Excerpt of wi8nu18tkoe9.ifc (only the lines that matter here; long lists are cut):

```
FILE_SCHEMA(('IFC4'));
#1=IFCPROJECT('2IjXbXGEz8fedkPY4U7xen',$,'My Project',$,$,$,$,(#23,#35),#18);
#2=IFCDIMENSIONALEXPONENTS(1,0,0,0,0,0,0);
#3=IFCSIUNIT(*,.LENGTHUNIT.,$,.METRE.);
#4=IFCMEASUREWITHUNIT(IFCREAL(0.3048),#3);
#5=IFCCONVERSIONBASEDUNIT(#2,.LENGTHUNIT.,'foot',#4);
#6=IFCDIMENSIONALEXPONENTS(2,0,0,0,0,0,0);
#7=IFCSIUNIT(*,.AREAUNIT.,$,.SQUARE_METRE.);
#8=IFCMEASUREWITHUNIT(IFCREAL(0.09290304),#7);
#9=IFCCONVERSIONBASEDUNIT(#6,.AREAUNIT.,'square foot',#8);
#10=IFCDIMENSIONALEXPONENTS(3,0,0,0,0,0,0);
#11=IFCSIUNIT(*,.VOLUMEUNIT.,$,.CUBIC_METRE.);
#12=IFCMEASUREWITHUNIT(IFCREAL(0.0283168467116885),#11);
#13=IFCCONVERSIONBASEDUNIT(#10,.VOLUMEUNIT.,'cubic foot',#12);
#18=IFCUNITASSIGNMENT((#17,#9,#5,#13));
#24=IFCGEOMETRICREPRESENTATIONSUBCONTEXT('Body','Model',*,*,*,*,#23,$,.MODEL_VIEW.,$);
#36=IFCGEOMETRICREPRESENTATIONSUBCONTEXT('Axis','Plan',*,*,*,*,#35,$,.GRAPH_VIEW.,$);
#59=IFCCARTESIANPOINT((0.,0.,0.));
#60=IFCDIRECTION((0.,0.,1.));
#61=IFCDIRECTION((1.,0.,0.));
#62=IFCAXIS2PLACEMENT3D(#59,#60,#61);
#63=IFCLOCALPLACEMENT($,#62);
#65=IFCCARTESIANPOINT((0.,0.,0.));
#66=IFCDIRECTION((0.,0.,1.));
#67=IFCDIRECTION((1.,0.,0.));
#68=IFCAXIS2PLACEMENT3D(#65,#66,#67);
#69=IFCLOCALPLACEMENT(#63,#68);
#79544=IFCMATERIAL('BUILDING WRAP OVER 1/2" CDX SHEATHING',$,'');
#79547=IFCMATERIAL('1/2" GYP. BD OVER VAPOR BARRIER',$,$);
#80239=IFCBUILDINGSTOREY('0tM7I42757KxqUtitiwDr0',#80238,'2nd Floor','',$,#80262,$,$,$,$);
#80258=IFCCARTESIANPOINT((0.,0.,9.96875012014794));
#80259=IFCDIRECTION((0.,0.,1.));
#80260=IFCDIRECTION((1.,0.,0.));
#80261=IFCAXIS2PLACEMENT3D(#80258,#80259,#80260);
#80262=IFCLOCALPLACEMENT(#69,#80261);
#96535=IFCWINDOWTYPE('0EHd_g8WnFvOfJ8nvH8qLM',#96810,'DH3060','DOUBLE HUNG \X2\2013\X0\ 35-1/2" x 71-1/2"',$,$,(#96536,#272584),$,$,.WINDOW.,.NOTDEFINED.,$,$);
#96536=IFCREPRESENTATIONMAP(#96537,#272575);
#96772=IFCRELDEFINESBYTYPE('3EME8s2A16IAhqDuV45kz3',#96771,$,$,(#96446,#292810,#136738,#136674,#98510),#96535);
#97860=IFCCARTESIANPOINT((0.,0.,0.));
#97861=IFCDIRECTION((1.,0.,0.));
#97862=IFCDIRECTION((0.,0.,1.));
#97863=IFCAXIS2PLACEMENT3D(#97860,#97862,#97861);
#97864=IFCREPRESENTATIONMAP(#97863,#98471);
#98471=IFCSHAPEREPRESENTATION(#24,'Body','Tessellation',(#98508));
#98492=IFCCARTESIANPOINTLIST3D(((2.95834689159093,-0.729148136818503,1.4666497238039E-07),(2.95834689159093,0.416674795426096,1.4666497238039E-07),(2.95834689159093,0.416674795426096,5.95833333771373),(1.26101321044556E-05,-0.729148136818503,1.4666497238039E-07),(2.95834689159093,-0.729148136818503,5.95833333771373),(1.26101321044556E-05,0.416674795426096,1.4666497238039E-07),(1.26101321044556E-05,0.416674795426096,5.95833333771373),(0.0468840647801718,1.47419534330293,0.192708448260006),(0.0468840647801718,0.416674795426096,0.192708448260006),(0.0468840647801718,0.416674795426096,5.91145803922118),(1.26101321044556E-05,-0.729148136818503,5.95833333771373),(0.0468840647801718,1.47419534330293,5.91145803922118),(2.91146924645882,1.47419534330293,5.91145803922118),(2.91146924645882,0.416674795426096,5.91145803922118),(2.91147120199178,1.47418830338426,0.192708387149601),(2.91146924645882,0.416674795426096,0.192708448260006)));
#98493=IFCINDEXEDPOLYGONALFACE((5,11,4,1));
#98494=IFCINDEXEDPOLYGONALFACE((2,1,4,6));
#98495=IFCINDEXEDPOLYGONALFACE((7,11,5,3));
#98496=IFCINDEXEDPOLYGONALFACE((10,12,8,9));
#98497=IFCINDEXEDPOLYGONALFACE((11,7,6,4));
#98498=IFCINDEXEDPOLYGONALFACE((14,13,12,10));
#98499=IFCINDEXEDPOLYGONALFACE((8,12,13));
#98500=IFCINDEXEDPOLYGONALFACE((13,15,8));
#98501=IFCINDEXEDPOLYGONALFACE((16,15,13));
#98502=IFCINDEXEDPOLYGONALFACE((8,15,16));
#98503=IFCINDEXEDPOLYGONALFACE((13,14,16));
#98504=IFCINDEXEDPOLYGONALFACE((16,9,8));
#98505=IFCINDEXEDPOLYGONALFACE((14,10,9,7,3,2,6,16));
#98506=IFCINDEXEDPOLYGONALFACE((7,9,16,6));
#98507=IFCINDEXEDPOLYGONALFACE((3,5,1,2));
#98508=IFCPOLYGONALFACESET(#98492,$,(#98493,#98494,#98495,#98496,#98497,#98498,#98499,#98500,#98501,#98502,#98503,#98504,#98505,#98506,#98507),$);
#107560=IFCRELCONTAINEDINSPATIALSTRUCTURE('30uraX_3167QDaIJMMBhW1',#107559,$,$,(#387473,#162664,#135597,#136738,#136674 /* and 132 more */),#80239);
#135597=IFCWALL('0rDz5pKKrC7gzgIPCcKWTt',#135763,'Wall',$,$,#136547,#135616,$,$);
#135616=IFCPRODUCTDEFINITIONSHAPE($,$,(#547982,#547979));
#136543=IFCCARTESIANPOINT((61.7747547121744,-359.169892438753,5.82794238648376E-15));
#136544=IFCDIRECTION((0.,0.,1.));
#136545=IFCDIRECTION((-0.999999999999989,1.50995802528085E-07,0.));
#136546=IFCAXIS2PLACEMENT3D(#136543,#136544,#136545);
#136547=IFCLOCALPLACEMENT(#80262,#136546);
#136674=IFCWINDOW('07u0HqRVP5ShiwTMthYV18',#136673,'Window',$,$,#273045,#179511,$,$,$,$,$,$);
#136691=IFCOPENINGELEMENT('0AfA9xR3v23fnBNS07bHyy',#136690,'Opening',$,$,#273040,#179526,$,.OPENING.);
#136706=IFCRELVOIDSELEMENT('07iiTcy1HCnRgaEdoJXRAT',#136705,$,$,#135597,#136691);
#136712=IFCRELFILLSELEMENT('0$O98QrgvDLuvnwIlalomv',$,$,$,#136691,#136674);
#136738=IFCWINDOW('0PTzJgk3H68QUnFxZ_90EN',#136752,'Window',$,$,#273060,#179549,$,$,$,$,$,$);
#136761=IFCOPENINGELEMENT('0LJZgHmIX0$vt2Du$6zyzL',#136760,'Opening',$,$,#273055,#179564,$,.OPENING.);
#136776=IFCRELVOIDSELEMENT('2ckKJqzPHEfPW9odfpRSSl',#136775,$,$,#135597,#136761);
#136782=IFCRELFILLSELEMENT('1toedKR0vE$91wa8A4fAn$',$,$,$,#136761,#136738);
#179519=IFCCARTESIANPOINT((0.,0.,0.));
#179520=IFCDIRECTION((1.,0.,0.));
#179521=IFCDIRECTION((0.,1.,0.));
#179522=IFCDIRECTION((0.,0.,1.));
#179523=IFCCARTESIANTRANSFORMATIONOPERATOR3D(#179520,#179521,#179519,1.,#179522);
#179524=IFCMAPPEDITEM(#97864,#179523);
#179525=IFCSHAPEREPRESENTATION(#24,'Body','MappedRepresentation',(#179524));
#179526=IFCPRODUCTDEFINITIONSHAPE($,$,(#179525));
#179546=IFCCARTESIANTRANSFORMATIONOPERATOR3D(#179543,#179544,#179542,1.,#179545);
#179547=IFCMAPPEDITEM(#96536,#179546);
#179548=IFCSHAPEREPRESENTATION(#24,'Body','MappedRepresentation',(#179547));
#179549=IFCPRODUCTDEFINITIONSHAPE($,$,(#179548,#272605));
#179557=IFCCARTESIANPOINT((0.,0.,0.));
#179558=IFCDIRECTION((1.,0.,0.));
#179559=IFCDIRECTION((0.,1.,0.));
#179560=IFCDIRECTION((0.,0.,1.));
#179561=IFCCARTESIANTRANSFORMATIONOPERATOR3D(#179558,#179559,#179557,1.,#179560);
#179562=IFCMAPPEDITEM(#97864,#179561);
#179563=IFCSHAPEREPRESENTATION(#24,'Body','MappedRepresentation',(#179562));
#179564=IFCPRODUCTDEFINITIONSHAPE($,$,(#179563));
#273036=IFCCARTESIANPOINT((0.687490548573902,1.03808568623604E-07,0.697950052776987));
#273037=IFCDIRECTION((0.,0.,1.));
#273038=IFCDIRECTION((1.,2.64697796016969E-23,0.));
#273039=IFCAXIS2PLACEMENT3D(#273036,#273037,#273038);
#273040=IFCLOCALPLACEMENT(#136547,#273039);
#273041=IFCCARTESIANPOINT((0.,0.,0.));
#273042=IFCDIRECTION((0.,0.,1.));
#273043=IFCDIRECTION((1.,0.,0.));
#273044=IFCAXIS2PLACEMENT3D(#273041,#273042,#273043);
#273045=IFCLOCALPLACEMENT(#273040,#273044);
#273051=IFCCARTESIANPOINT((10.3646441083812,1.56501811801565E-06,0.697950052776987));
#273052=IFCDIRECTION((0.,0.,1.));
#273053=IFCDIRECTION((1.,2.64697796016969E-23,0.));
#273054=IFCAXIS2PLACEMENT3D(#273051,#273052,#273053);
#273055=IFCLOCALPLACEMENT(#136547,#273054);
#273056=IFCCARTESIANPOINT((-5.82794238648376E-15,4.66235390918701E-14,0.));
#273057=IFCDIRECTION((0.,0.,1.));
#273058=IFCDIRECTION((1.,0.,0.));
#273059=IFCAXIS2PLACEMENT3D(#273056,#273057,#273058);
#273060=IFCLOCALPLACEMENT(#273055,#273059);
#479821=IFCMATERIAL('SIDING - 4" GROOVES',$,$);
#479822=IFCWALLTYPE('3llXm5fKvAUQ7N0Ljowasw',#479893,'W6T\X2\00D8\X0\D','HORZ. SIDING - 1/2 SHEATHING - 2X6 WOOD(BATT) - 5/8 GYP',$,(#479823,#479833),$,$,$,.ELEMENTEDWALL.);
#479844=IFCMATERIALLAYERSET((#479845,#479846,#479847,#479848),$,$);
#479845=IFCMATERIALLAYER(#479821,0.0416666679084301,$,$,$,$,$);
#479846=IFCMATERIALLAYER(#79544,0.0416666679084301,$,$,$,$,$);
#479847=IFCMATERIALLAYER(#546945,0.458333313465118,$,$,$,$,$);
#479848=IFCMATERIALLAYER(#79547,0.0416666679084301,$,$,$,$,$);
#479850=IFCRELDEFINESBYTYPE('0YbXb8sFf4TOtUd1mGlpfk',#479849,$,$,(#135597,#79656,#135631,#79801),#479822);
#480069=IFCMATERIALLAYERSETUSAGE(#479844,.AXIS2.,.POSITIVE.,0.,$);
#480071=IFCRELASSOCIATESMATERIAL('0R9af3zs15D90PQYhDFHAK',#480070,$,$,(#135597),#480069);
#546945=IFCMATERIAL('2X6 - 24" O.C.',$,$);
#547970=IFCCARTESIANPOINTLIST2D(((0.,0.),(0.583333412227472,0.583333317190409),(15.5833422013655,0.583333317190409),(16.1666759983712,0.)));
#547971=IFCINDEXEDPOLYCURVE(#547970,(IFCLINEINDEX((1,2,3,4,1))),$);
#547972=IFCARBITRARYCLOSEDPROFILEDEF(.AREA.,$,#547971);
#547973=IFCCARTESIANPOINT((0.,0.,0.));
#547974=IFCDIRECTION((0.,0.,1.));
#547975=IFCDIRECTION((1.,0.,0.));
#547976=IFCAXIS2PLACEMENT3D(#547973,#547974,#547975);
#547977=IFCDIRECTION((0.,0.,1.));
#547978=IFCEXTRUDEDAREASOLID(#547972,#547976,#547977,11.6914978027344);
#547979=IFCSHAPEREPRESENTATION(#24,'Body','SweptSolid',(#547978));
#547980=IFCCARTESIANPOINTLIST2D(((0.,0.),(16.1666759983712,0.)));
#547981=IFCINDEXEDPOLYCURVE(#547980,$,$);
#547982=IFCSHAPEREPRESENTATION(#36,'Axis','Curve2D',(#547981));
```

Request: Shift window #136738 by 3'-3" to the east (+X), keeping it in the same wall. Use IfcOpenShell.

```python
import ifcopenshell
import ifcopenshell.api.geometry
import ifcopenshell.util.placement
import ifcopenshell.util.unit

model = ifcopenshell.open("wi8nu18tkoe9.ifc")
unit_scale = ifcopenshell.util.unit.calculate_unit_scale(model)

window = model.by_id(136738)
opening = window.FillsVoids[0].RelatingOpeningElement
wall = opening.VoidsElements[0].RelatingBuildingElement

wall_matrix = ifcopenshell.util.placement.get_local_placement(wall.ObjectPlacement)
shift = wall_matrix[:3, 0] * -39 * 0.0254 / unit_scale
before = ifcopenshell.util.placement.get_local_placement(window.ObjectPlacement)[:3, 3].copy()

# The window is placed relative to its opening, so it follows when the opening moves.
matrix = ifcopenshell.util.placement.get_local_placement(opening.ObjectPlacement)
matrix[:3, 3] += shift
ifcopenshell.api.geometry.edit_object_placement(
    model, product=opening, matrix=matrix, is_si=False, should_transform_children=True
)

after = ifcopenshell.util.placement.get_local_placement(window.ObjectPlacement)[:3, 3]
print("window moved by", (after - before).round(3) + 0.0)

model.write("wi8nu18tkoe9_v2.ifc")
```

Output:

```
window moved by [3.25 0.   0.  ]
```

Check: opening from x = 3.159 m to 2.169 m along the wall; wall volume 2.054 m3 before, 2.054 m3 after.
